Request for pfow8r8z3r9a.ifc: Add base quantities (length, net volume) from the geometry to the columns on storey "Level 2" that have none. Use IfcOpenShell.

First a look at what the model holds.

```python
import ifcopenshell
import ifcopenshell.util.element
import ifcopenshell.util.unit

model = ifcopenshell.open("pfow8r8z3r9a.ifc")
print(model.schema)
for unit_type in ("LENGTHUNIT", "AREAUNIT", "VOLUMEUNIT"):
    print(unit_type, ifcopenshell.util.unit.calculate_unit_scale(model, unit_type))
storey = next(s for s in model.by_type("IfcBuildingStorey") if s.Name == "Level 2")
columns = [e for e in ifcopenshell.util.element.get_decomposition(storey) if e.is_a("IfcColumn")]
for e in sorted(columns, key=lambda e: e.id()):
    print(e.id(), e.is_a(), e.Name, list(ifcopenshell.util.element.get_psets(e, qtos_only=True)), sep=" | ")
```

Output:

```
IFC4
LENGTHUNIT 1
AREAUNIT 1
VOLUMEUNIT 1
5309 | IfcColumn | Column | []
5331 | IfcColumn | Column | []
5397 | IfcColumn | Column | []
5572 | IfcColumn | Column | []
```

```python
import ifcopenshell
import ifcopenshell.api.pset
import ifcopenshell.geom
import ifcopenshell.util.element
import ifcopenshell.util.shape
import ifcopenshell.util.unit

model = ifcopenshell.open("pfow8r8z3r9a.ifc")
unit_scale = ifcopenshell.util.unit.calculate_unit_scale(model)
volume_scale = ifcopenshell.util.unit.calculate_unit_scale(model, "VOLUMEUNIT")
settings = ifcopenshell.geom.settings()

storey = next(s for s in model.by_type("IfcBuildingStorey") if s.Name == "Level 2")
columns = [e for e in ifcopenshell.util.element.get_decomposition(storey) if e.is_a("IfcColumn")]

for e in sorted(columns, key=lambda e: e.id()):
    if ifcopenshell.util.element.get_psets(e, qtos_only=True, should_inherit=False):
        continue
    # Geometry comes back in metres, in the element's own axes.
    shape = ifcopenshell.geom.create_shape(settings, e)
    values = {
        "Length": ifcopenshell.util.shape.get_z(shape.geometry) / unit_scale,
        "NetVolume": ifcopenshell.util.shape.get_volume(shape.geometry) / volume_scale,
    }
    qto = ifcopenshell.api.pset.add_qto(model, product=e, name="Qto_ColumnBaseQuantities")
    ifcopenshell.api.pset.edit_qto(model, qto=qto, properties=values)
    print(e.id(), {k: round(v, 3) for k, v in values.items()})

model.write("pfow8r8z3r9a-out.ifc")
```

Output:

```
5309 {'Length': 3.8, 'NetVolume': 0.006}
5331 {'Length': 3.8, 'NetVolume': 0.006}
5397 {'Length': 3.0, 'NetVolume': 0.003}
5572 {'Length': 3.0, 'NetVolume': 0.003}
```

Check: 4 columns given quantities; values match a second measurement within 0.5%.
